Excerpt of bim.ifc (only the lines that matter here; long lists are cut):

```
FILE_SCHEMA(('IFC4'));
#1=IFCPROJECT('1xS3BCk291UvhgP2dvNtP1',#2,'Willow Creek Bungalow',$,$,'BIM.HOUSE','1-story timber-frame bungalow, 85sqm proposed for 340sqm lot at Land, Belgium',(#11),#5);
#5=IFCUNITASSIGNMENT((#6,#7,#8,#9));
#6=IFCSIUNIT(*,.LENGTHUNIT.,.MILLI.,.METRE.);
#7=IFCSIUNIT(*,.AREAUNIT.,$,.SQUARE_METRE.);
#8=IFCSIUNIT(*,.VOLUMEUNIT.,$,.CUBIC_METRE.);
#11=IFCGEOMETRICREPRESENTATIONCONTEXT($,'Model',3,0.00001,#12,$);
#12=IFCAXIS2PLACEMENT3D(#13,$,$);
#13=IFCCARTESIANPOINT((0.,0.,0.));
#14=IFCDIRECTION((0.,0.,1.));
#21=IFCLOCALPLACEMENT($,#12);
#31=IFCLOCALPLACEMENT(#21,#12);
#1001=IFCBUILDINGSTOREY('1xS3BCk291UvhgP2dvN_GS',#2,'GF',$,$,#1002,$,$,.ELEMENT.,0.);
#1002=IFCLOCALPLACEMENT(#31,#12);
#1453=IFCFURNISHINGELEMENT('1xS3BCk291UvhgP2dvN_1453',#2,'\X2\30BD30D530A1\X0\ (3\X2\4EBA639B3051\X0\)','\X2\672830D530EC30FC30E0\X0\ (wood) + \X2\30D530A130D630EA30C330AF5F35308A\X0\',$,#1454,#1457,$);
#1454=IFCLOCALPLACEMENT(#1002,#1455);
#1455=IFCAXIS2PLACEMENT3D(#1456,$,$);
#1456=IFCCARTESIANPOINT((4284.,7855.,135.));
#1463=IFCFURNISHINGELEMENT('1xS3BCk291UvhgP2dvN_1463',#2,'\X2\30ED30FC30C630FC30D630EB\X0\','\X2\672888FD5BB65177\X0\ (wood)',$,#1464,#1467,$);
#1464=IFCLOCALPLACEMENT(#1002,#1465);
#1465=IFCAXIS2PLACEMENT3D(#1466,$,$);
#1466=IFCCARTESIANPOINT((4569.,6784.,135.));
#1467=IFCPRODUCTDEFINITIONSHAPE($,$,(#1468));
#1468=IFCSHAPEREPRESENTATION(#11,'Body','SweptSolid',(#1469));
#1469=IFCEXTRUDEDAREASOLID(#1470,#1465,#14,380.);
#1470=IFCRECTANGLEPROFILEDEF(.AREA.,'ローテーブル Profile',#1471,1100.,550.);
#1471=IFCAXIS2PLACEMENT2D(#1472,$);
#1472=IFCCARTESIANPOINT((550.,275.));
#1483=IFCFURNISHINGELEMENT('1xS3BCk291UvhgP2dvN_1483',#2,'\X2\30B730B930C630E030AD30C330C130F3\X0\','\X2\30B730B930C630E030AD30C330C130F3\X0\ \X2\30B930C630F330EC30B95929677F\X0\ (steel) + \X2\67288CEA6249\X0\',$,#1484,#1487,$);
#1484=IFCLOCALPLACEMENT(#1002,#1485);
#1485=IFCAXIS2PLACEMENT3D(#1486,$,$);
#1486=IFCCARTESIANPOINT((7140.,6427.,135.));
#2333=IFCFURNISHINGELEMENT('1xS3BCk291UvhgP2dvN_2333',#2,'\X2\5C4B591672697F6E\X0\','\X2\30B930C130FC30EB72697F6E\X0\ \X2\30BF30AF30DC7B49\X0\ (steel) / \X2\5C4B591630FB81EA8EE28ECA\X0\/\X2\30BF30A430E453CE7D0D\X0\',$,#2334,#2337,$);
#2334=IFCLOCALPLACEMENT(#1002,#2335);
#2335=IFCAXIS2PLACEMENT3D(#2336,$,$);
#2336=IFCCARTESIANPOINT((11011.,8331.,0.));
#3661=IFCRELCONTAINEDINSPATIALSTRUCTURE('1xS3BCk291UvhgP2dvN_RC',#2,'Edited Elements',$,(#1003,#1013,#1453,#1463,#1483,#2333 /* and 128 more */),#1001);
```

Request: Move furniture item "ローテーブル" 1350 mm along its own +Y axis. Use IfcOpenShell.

```python
import ifcopenshell
import ifcopenshell.api.geometry
import ifcopenshell.util.placement
import ifcopenshell.util.unit

model = ifcopenshell.open("bim.ifc")
unit_scale = ifcopenshell.util.unit.calculate_unit_scale(model)

item = model.by_guid("1xS3BCk291UvhgP2dvN_1463")
matrix = ifcopenshell.util.placement.get_local_placement(item.ObjectPlacement)
matrix[:3, 3] += matrix[:3, 1] * 1.35 / unit_scale
ifcopenshell.api.geometry.edit_object_placement(model, product=item, matrix=matrix, is_si=False)

print(ifcopenshell.util.placement.get_local_placement(item.ObjectPlacement).round(3) + 0.0)

model.write("bim_edited.ifc")
```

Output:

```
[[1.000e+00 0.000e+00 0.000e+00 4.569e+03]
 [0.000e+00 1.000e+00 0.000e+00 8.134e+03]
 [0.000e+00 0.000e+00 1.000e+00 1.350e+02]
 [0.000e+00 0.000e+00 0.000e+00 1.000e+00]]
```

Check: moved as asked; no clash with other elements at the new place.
